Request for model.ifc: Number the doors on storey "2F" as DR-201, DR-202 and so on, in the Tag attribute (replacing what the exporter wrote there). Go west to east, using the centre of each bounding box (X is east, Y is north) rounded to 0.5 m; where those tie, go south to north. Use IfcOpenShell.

First a look at what the model holds.

```python
import ifcopenshell
import ifcopenshell.util.element
import ifcopenshell.util.placement

model = ifcopenshell.open("model.ifc")
print(model.schema)
storey = next(s for s in model.by_type("IfcBuildingStorey") if s.Name == "2F")
doors = [e for e in ifcopenshell.util.element.get_decomposition(storey) if e.is_a("IfcDoor")]
for e in sorted(doors, key=lambda e: e.id()):
    origin = ifcopenshell.util.placement.get_local_placement(e.ObjectPlacement)[:3, 3]
    print(e.id(), e.Tag, e.Name, origin.round(2) + 0.0, sep=" | ")
```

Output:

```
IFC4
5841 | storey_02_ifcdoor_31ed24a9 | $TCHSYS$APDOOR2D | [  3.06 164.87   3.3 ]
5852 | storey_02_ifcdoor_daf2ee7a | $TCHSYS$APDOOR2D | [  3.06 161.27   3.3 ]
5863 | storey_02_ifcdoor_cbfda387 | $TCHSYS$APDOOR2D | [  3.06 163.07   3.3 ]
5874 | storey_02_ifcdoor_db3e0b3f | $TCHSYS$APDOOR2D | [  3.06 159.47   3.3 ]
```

```python
import ifcopenshell
import ifcopenshell.geom
import ifcopenshell.util.element
import ifcopenshell.util.shape

model = ifcopenshell.open("model.ifc")
settings = ifcopenshell.geom.settings()
settings.set("use-world-coords", True)


def centre(element):
    shape = ifcopenshell.geom.create_shape(settings, element)
    return ifcopenshell.util.shape.get_bbox_centroid(shape.geometry)


storey = next(s for s in model.by_type("IfcBuildingStorey") if s.Name == "2F")
doors = [e for e in ifcopenshell.util.element.get_decomposition(storey) if e.is_a("IfcDoor")]

# Insertion points can sit at a corner or the storey origin, so sort by the geometry (in metres).
centres = {e: centre(e) for e in doors}
doors.sort(key=lambda e: (round(centres[e][0] / 0.5), centres[e][1]))

for i, e in enumerate(doors, start=1):
    number = f"DR-2{i:02d}"
    e.Tag = number
    print(e.id(), number)

model.write("model_edited.ifc")
```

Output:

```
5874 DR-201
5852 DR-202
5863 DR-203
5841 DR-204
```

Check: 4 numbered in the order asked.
